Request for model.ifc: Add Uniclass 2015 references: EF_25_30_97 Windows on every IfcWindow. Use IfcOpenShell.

First a look at what the model holds.

```python
import ifcopenshell

model = ifcopenshell.open("model.ifc")
print(model.schema)
print("classifications:", [c.Name for c in model.by_type("IfcClassification")])
for ifc_class in ("IfcDoor", "IfcRoof", "IfcStair", "IfcWall", "IfcWindow"):
    print(ifc_class, len(model.by_type(ifc_class)))
```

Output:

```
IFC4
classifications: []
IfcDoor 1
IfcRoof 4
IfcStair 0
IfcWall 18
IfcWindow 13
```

```python
import ifcopenshell
import ifcopenshell.api.classification

model = ifcopenshell.open("model.ifc")

system = ifcopenshell.api.classification.add_classification(model, classification="Uniclass 2015")

codes = {
    "IfcWindow": ("EF_25_30_97", "Windows"),
}
for ifc_class, (code, name) in codes.items():
    products = model.by_type(ifc_class)
    ifcopenshell.api.classification.add_reference(
        model, products=products, classification=system, identification=code, name=name
    )
    print(code, len(products))

model.write("model_edited.ifc")
```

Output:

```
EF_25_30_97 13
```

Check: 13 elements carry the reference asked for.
